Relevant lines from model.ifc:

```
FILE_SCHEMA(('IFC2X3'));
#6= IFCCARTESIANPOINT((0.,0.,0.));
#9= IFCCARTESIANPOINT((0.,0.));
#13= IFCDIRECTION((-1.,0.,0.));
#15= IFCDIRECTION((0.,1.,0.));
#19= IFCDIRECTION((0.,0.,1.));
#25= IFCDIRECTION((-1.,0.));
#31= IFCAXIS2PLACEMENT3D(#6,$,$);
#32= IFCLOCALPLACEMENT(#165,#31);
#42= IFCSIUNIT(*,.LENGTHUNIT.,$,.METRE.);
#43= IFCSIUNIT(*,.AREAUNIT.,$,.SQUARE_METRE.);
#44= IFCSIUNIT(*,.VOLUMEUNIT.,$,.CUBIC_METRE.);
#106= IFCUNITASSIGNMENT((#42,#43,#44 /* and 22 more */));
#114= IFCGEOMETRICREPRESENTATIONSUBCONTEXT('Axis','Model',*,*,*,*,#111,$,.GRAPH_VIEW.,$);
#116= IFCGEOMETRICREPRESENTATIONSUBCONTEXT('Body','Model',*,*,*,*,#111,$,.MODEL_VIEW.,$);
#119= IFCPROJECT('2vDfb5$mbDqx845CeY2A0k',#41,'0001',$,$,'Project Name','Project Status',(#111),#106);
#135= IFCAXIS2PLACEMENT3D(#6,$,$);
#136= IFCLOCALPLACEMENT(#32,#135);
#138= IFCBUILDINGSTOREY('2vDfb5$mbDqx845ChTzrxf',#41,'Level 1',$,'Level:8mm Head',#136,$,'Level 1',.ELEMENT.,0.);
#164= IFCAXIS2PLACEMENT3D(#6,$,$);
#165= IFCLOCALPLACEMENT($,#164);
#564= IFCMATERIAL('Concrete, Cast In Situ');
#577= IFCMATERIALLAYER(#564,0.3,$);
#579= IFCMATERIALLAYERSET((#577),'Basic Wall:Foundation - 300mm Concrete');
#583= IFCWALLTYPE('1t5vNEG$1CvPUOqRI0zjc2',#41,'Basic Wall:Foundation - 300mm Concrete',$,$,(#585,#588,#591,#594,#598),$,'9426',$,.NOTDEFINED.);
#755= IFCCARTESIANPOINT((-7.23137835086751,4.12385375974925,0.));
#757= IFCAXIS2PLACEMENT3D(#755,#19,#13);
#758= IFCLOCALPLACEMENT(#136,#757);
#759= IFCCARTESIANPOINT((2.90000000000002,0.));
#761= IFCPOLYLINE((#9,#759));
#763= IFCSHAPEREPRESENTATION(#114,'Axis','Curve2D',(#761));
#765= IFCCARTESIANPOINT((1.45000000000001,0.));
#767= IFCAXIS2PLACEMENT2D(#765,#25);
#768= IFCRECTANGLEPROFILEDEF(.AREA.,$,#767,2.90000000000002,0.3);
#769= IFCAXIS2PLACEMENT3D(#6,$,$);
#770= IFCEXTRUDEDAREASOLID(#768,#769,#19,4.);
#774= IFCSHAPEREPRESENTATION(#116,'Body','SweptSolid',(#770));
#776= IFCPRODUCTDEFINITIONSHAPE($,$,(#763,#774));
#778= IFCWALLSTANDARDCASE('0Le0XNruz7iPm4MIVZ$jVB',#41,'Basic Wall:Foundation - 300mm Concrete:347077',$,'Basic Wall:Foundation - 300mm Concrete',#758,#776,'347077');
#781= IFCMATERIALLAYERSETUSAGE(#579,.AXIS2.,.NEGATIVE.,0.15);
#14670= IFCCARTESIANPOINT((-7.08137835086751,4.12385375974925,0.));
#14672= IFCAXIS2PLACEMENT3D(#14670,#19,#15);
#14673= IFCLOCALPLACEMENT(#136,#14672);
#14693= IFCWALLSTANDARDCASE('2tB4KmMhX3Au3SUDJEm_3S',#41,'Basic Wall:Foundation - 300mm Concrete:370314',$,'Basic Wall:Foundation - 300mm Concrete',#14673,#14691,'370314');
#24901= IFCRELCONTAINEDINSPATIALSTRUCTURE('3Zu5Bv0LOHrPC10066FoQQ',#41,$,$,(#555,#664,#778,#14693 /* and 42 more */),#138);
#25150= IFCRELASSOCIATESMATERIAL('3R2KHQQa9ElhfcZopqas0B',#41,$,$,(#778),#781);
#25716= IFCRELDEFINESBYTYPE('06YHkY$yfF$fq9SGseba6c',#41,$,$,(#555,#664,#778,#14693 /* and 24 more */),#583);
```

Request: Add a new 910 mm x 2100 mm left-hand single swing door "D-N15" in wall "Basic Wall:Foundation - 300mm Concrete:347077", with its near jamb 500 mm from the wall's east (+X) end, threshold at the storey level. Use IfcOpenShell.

```python
import numpy as np
import ifcopenshell
import ifcopenshell.api.feature
import ifcopenshell.api.geometry
import ifcopenshell.api.root
import ifcopenshell.api.spatial
import ifcopenshell.api.type
import ifcopenshell.geom
import ifcopenshell.util.element
import ifcopenshell.util.placement
import ifcopenshell.util.representation
import ifcopenshell.util.shape
import ifcopenshell.util.unit

model = ifcopenshell.open("model.ifc")
unit_scale = ifcopenshell.util.unit.calculate_unit_scale(model)
settings = ifcopenshell.geom.settings()


def volume(element):
    """Net volume in cubic metres, openings subtracted."""
    shape = ifcopenshell.geom.create_shape(settings, element)
    return ifcopenshell.util.shape.get_volume(shape.geometry)


wall = model.by_guid("0Le0XNruz7iPm4MIVZ$jVB")
storey = ifcopenshell.util.element.get_container(wall, ifc_class="IfcBuildingStorey")
context = ifcopenshell.util.representation.get_context(model, "Model", "Body", "MODEL_VIEW")
before = volume(wall)

width, height, from_end, sill = 0.91, 2.1, 0.5, 0.0  # metres

# The wall runs along its own X axis, and the end named is its -X end.
wall_shape = ifcopenshell.geom.create_shape(settings, wall)
x, y, z = ifcopenshell.util.shape.get_vertices(wall_shape.geometry).T
start = x.min() + from_end
face, thickness = float(y.min()), float(y.max() - y.min())
wall_matrix = ifcopenshell.util.placement.get_local_placement(wall.ObjectPlacement)
level = ifcopenshell.util.placement.get_local_placement(storey.ObjectPlacement)[2, 3]


def in_wall(x, y):
    """Placement at x, y metres in the wall's axes, at sill height."""
    matrix = wall_matrix.copy()
    matrix[:, 3] = wall_matrix @ np.array([x / unit_scale, y / unit_scale, 0.0, 1.0])
    matrix[2, 3] = level + sill / unit_scale
    return matrix


# Opening: a box that overshoots both wall faces by 50 mm.
opening = ifcopenshell.api.root.create_entity(model, ifc_class="IfcOpeningElement")
box = ifcopenshell.api.geometry.add_wall_representation(
    model, context=context, length=width, height=height, thickness=thickness + 0.1
)
ifcopenshell.api.geometry.assign_representation(model, product=opening, representation=box)
ifcopenshell.api.geometry.edit_object_placement(model, product=opening, matrix=in_wall(start, face - 0.05), is_si=False)
ifcopenshell.api.feature.add_feature(model, feature=opening, element=wall)

door = ifcopenshell.api.root.create_entity(model, ifc_class="IfcDoor", name="D-N15")
door.OverallWidth, door.OverallHeight = width / unit_scale, height / unit_scale
body = ifcopenshell.api.geometry.add_door_representation(
    model,
    context=context,
    overall_width=door.OverallWidth,
    overall_height=door.OverallHeight,
    operation_type="SINGLE_SWING_LEFT",
    lining_properties={"LiningDepth": thickness / unit_scale, "ThresholdDepth": thickness / unit_scale},
)
ifcopenshell.api.geometry.assign_representation(model, product=door, representation=body)
ifcopenshell.api.spatial.assign_container(model, products=[door], relating_structure=storey)
fills = ifcopenshell.api.feature.add_filling(model, opening=opening, element=door)
fills.OwnerHistory = door.OwnerHistory  # required in IFC2X3

# IFC2X3 keeps the operation on the door style.
style = ifcopenshell.api.root.create_entity(model, ifc_class="IfcDoorStyle", name="D-N15")
style.OperationType, style.ConstructionType = "SINGLE_SWING_LEFT", "NOTDEFINED"
style.ParameterTakesPrecedence = style.Sizeable = False
ifcopenshell.api.type.assign_type(model, related_objects=[door], relating_type=style)

# The lining spans the wall, so the door starts at the wall face.
ifcopenshell.api.geometry.edit_object_placement(model, product=door, matrix=in_wall(start, face), is_si=False)

after = volume(wall)

print(f"wall volume {before:.3f} -> {after:.3f} m3")

model.write("model_edited.ifc")
```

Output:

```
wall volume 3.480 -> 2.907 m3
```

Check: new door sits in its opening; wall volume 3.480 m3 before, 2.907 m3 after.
